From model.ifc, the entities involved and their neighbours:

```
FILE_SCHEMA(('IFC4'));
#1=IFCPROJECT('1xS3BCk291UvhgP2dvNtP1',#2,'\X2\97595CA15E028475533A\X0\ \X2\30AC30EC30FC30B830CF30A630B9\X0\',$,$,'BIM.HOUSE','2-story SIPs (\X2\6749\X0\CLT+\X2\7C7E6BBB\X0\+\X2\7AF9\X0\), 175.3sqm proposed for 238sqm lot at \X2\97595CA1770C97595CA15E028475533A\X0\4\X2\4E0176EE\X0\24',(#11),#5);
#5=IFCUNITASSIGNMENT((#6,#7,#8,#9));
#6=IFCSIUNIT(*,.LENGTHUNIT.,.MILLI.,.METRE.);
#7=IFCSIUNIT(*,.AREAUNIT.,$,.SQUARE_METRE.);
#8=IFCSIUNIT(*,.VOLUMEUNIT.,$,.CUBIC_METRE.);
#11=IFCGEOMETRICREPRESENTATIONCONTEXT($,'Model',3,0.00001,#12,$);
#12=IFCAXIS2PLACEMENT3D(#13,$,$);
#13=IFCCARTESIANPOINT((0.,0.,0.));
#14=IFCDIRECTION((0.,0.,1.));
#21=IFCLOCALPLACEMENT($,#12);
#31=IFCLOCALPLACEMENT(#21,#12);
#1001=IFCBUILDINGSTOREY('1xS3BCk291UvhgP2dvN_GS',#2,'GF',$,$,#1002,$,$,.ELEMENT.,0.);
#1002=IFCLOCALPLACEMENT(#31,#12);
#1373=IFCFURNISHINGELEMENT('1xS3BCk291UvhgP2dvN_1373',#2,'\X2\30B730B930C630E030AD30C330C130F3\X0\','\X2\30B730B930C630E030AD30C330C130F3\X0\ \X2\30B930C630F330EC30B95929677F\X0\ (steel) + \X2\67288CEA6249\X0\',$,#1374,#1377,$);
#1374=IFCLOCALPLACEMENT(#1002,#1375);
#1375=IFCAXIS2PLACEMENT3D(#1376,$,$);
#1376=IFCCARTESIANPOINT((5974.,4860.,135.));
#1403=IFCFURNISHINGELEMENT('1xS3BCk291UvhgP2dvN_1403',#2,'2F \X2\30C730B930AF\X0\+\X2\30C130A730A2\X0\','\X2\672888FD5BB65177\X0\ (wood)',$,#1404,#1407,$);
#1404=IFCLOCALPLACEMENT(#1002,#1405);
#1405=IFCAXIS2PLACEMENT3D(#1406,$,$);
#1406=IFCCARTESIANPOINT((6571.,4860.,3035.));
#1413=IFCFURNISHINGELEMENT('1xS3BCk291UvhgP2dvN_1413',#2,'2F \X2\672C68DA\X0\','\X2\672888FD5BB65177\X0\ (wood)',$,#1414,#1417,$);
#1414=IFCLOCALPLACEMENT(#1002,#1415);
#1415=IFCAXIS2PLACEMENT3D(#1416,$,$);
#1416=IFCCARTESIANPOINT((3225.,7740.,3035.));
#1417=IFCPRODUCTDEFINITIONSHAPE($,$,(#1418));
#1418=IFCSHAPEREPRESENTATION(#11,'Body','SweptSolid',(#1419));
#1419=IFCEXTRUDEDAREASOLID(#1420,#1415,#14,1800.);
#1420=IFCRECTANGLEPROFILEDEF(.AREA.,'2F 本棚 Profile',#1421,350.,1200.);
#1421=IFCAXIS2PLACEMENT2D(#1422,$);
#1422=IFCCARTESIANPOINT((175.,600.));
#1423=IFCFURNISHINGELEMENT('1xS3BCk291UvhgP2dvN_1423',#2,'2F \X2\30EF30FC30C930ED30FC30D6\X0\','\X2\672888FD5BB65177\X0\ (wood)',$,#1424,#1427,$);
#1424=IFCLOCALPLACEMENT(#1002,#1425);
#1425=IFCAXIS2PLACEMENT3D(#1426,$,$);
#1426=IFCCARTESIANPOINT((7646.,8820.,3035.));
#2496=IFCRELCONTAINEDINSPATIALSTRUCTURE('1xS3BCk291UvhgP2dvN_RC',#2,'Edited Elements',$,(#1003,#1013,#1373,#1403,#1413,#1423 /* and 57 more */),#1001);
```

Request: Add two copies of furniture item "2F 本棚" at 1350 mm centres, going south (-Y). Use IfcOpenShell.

```python
import numpy as np
import ifcopenshell
import ifcopenshell.api.geometry
import ifcopenshell.api.root
import ifcopenshell.util.element
import ifcopenshell.util.placement
import ifcopenshell.util.unit

model = ifcopenshell.open("model.ifc")
unit_scale = ifcopenshell.util.unit.calculate_unit_scale(model)


def reuse_history(source, copy):
    """copy_class also copies each property set's owner history, people and application; keep the originals."""
    for rel in copy.IsDefinedBy:
        if rel.is_a("IfcRelDefinesByProperties") and (history := rel.RelatingPropertyDefinition.OwnerHistory):
            rel.RelatingPropertyDefinition.OwnerHistory = source.OwnerHistory
            ifcopenshell.util.element.remove_deep2(model, history)


source = model.by_id(1413)
base = ifcopenshell.util.placement.get_local_placement(source.ObjectPlacement)
step = np.array([0.0, -1.0, 0.0]) * 1.35 / unit_scale

for i in range(1, 3):
    copy = ifcopenshell.api.root.copy_class(model, product=source)
    copy.Representation = ifcopenshell.util.element.copy_deep(
        model, source.Representation, exclude=["IfcGeometricRepresentationContext", "IfcRepresentationMap"]
    )
    reuse_history(source, copy)
    matrix = base.copy()
    matrix[:3, 3] += i * step
    print("added at", matrix[:3, 3].round(3) + 0.0)
    ifcopenshell.api.geometry.edit_object_placement(model, product=copy, matrix=matrix, is_si=False)

model.write("model-out.ifc")
```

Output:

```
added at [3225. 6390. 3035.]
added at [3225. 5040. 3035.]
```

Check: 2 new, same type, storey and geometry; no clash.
